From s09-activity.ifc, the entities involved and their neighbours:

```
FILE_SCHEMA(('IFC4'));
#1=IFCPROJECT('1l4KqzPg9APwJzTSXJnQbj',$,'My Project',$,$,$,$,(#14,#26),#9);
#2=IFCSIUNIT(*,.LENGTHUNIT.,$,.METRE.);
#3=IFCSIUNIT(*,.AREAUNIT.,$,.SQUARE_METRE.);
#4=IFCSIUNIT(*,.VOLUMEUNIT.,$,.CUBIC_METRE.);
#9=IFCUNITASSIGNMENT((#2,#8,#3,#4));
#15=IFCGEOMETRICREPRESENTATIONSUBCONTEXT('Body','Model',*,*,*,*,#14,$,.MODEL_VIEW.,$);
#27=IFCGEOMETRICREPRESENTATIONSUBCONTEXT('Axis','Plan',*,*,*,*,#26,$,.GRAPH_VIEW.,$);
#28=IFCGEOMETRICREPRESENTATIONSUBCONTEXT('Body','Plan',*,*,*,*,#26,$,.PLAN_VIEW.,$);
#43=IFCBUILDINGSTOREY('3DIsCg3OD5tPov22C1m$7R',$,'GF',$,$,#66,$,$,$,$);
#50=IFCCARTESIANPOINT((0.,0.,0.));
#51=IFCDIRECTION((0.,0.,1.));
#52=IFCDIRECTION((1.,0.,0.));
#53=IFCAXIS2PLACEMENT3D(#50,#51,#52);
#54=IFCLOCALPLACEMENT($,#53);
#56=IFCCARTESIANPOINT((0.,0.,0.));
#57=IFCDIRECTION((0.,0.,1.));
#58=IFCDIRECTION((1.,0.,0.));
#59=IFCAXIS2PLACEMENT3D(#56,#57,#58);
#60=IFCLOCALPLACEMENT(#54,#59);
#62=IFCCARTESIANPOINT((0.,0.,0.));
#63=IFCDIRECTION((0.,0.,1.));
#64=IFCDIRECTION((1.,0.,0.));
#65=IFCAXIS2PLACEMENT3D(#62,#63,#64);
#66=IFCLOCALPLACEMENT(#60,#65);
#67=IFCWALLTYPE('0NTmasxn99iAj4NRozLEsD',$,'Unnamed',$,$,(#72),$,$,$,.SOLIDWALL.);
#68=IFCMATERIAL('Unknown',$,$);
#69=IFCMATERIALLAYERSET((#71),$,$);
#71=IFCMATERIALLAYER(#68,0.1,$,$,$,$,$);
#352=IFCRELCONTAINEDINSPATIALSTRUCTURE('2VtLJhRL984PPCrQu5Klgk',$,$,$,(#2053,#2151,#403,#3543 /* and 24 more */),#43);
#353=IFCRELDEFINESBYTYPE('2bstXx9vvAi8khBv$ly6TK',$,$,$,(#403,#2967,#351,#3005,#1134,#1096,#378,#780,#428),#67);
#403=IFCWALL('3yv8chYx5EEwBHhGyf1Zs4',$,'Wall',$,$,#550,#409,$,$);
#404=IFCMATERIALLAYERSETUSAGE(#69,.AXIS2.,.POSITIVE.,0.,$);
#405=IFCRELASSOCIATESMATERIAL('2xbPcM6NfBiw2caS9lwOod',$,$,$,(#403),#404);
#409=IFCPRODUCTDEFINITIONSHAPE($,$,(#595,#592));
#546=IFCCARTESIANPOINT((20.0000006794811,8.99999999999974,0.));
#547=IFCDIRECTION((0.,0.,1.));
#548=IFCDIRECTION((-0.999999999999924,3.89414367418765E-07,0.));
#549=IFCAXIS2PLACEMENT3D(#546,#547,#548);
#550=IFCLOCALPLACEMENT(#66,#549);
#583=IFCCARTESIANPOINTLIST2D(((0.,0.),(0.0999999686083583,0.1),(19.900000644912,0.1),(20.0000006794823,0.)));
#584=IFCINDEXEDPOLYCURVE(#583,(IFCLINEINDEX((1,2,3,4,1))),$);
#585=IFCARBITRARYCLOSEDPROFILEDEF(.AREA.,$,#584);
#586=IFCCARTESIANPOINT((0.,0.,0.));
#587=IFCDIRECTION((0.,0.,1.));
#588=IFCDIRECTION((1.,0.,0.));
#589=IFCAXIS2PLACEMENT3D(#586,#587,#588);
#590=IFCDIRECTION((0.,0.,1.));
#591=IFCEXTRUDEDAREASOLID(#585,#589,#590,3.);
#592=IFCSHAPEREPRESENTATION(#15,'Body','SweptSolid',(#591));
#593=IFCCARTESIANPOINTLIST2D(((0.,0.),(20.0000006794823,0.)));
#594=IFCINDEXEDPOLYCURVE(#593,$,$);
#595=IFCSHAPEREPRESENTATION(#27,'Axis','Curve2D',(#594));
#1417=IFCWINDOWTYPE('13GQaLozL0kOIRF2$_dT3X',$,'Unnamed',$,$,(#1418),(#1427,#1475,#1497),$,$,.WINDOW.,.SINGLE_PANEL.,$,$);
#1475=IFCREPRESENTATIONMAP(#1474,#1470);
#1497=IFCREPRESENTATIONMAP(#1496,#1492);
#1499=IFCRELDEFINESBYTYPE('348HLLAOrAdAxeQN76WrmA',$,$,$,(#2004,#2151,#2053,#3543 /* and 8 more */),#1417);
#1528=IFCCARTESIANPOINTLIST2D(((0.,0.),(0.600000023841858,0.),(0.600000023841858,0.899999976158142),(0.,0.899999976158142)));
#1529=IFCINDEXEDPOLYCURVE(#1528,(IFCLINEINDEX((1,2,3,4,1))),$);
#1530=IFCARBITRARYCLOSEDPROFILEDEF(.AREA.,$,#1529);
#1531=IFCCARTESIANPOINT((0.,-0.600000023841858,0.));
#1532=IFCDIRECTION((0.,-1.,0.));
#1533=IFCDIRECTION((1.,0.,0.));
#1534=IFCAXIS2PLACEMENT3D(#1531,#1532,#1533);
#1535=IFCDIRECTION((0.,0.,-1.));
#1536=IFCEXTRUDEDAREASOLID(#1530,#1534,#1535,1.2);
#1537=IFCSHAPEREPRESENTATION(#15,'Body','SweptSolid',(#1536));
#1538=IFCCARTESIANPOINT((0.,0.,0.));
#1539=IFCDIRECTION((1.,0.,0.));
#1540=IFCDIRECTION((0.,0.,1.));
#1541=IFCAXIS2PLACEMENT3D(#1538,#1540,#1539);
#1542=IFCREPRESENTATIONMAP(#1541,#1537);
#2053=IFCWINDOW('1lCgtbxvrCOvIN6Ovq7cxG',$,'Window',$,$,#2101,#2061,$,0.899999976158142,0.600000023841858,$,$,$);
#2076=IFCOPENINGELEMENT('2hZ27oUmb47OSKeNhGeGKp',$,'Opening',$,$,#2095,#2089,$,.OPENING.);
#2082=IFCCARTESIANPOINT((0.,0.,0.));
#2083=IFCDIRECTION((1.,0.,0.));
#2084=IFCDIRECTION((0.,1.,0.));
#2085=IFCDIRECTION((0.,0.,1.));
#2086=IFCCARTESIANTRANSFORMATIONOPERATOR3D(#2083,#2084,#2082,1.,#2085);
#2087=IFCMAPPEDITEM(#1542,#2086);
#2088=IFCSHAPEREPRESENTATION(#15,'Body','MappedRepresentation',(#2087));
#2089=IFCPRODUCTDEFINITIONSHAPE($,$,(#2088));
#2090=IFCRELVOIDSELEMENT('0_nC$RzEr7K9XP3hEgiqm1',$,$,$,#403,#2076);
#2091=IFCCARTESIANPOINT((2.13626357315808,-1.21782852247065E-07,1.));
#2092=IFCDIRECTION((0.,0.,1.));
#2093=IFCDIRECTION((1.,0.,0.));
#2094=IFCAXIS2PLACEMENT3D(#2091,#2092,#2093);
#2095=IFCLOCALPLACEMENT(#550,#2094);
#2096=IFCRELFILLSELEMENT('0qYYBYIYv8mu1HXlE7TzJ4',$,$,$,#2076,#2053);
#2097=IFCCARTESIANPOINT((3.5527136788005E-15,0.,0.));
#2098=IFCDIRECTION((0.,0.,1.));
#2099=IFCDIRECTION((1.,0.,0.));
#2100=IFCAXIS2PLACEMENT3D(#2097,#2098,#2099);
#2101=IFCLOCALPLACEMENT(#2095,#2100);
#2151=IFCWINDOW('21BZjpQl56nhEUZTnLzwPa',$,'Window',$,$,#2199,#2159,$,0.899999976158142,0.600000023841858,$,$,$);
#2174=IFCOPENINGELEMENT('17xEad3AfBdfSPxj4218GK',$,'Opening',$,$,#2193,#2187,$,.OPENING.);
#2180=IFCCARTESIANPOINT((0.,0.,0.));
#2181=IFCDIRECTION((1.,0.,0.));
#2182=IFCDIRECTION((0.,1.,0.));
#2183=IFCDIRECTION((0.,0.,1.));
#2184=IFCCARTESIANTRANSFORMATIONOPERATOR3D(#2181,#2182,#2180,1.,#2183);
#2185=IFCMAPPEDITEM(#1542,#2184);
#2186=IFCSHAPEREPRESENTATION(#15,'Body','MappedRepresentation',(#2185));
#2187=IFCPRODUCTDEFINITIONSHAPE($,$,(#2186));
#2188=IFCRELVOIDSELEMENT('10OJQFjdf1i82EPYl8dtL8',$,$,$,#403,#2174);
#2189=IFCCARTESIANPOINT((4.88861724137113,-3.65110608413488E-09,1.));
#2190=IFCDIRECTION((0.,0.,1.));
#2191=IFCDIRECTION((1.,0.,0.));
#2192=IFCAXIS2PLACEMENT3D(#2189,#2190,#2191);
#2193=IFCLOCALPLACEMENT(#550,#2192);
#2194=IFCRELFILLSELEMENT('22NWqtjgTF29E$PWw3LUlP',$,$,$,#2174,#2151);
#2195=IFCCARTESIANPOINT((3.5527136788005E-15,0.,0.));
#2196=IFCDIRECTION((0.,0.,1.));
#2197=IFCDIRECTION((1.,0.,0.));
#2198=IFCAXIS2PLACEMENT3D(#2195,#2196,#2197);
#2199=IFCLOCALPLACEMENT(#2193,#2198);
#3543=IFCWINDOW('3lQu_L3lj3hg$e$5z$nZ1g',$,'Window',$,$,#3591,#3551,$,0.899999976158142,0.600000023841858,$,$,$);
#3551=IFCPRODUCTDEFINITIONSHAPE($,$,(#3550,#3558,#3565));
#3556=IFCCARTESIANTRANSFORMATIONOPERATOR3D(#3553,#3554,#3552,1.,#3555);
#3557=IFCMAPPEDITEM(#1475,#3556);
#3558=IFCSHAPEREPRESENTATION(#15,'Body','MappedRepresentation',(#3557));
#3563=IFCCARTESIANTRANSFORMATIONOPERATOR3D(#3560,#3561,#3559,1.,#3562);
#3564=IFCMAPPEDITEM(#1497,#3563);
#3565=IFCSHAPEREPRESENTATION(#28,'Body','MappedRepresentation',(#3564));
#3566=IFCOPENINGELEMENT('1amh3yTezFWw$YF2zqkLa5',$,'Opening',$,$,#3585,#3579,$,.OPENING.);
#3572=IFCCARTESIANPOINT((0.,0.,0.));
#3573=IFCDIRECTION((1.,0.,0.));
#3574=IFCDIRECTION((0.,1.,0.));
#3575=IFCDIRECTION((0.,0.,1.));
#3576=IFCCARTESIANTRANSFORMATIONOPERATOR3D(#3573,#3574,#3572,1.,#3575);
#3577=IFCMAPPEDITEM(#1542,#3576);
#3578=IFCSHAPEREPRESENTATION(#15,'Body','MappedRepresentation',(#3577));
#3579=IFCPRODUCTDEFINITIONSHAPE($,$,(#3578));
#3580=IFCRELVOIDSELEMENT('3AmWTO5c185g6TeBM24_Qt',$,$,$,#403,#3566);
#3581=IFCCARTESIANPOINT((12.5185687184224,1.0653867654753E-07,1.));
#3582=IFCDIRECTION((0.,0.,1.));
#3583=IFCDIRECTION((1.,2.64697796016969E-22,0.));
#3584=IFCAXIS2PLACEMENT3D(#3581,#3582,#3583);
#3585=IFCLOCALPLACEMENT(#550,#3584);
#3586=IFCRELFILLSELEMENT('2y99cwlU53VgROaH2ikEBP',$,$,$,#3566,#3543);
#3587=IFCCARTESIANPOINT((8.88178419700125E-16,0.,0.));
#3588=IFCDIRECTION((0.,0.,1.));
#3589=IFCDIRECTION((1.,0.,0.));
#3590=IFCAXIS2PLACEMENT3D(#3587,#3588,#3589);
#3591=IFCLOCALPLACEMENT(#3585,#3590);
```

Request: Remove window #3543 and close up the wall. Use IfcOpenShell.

```python
import ifcopenshell
import ifcopenshell.api.feature
import ifcopenshell.api.root
import ifcopenshell.geom
import ifcopenshell.util.shape

model = ifcopenshell.open("s09-activity.ifc")
settings = ifcopenshell.geom.settings()


def volume(element):
    """Net volume in cubic metres, openings subtracted."""
    shape = ifcopenshell.geom.create_shape(settings, element)
    return ifcopenshell.util.shape.get_volume(shape.geometry)


window = model.by_guid("3lQu_L3lj3hg$e$5z$nZ1g")
opening = window.FillsVoids[0].RelatingOpeningElement
wall = opening.VoidsElements[0].RelatingBuildingElement
before = volume(wall)

ifcopenshell.api.root.remove_product(model, product=window)
ifcopenshell.api.feature.remove_feature(model, feature=opening)

after = volume(wall)

print(f"wall volume {before:.3f} -> {after:.3f} m3")

model.write("s09-activity_v2.ifc")
```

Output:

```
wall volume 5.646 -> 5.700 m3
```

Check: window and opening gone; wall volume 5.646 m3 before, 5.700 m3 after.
